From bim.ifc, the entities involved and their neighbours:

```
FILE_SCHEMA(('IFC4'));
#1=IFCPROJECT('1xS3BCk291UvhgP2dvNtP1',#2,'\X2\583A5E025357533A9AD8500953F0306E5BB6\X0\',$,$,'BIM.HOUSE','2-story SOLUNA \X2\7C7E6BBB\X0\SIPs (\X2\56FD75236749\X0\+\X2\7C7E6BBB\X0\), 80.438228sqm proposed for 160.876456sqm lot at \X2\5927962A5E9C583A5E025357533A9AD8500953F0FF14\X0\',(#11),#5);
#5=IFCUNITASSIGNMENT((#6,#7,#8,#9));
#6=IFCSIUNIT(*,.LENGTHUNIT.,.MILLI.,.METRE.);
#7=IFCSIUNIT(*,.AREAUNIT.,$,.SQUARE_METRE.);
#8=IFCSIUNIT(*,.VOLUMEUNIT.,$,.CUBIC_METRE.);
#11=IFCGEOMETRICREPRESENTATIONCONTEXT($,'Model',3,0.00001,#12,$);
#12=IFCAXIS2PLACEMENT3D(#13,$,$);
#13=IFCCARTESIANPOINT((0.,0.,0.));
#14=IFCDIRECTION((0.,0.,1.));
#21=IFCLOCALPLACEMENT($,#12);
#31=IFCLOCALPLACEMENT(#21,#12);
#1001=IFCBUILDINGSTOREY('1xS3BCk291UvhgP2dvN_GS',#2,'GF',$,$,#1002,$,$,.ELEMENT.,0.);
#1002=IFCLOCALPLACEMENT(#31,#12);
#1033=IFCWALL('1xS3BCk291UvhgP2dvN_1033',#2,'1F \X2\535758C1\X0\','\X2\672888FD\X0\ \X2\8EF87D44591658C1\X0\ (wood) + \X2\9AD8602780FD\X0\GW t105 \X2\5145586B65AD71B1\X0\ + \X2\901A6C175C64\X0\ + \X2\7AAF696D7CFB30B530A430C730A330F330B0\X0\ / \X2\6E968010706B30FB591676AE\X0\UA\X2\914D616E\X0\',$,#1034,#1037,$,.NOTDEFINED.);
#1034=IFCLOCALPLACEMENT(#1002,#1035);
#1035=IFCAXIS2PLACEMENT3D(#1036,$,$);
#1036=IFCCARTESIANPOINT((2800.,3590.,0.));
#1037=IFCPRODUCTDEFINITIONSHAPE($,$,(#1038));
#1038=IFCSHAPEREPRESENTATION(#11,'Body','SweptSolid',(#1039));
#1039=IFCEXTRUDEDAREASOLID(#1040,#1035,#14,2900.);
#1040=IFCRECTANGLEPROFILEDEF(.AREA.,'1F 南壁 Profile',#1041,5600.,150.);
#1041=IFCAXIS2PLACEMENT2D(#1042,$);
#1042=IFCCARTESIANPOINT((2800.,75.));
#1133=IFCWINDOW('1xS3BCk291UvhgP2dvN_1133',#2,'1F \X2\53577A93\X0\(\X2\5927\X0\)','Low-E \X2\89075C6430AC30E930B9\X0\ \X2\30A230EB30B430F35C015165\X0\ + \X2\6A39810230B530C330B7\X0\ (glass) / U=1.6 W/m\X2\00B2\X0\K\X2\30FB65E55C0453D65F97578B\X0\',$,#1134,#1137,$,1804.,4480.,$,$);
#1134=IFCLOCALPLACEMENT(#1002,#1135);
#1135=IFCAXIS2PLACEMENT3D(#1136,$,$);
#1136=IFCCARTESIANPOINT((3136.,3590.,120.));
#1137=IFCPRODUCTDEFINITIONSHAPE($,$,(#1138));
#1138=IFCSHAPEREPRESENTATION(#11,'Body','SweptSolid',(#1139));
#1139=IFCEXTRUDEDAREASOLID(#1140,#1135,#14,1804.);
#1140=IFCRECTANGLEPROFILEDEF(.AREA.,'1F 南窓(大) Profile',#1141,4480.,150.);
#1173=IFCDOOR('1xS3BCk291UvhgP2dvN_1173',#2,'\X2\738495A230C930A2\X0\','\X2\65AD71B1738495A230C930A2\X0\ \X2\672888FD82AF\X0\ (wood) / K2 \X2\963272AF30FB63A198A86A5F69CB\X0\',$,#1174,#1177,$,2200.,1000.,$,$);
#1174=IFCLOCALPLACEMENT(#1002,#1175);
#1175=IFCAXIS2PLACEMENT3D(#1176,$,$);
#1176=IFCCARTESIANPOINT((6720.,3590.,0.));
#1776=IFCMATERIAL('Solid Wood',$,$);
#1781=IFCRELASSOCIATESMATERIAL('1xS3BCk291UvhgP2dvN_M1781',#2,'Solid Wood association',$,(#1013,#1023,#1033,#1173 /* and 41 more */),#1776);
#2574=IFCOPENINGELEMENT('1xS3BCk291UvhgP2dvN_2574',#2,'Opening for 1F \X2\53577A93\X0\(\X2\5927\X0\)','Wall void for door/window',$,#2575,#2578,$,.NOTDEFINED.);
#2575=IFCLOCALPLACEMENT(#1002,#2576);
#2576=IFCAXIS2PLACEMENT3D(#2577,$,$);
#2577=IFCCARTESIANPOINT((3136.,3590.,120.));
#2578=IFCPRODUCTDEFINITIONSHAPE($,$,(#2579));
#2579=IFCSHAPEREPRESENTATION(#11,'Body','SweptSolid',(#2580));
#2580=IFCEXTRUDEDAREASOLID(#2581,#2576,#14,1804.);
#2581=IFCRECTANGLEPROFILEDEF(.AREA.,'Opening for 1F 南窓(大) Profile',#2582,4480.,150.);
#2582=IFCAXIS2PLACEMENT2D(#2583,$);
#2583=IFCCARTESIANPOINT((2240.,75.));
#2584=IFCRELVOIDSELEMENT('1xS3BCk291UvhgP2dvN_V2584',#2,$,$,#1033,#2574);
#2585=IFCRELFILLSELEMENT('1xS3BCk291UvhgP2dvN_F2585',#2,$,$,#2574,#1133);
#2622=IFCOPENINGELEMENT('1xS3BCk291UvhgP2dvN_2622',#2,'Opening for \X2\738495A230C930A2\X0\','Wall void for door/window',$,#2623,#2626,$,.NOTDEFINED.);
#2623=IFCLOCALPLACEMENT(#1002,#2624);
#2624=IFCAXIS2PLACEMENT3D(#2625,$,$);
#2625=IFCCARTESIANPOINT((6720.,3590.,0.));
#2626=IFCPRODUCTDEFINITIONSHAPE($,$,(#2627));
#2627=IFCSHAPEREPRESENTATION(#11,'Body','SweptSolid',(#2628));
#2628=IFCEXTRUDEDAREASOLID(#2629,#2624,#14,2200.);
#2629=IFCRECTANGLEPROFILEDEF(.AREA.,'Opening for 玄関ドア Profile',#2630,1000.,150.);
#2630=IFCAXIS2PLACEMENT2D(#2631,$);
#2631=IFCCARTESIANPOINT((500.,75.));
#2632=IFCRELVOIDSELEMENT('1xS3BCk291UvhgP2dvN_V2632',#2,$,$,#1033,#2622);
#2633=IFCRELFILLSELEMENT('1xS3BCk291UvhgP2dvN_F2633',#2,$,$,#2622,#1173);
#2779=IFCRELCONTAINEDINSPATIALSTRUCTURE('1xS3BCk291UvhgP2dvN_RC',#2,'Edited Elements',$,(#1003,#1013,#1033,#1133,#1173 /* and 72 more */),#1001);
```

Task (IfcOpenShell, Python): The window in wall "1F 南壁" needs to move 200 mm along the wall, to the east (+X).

```python
import ifcopenshell
import ifcopenshell.api.geometry
import ifcopenshell.util.placement

model = ifcopenshell.open("bim.ifc")

window = model.by_id(1133)
opening = window.FillsVoids[0].RelatingOpeningElement
wall = opening.VoidsElements[0].RelatingBuildingElement

wall_matrix = ifcopenshell.util.placement.get_local_placement(wall.ObjectPlacement)
shift = wall_matrix[:3, 0] * 200.0
before = ifcopenshell.util.placement.get_local_placement(window.ObjectPlacement)[:3, 3].copy()

# The window is not placed relative to its opening, so move both.
for product in (opening, window):
    matrix = ifcopenshell.util.placement.get_local_placement(product.ObjectPlacement)
    matrix[:3, 3] += shift
    ifcopenshell.api.geometry.edit_object_placement(model, product=product, matrix=matrix, is_si=False)

after = ifcopenshell.util.placement.get_local_placement(window.ObjectPlacement)[:3, 3]
print("window moved by", (after - before).round(3) + 0.0)

model.write("bim_updated.ifc")
```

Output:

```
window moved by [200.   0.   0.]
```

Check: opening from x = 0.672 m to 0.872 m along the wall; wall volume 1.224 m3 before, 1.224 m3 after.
